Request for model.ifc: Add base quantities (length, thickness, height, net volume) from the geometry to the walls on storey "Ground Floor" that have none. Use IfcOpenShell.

First a look at what the model holds.

```python
import ifcopenshell
import ifcopenshell.util.element
import ifcopenshell.util.unit

model = ifcopenshell.open("model.ifc")
print(model.schema)
for unit_type in ("LENGTHUNIT", "AREAUNIT", "VOLUMEUNIT"):
    print(unit_type, ifcopenshell.util.unit.calculate_unit_scale(model, unit_type))
storey = next(s for s in model.by_type("IfcBuildingStorey") if s.Name == "Ground Floor")
walls = [e for e in ifcopenshell.util.element.get_decomposition(storey) if e.is_a("IfcWall")]
for e in sorted(walls, key=lambda e: e.id()):
    print(e.id(), e.is_a(), e.Name, list(ifcopenshell.util.element.get_psets(e, qtos_only=True)), sep=" | ")
```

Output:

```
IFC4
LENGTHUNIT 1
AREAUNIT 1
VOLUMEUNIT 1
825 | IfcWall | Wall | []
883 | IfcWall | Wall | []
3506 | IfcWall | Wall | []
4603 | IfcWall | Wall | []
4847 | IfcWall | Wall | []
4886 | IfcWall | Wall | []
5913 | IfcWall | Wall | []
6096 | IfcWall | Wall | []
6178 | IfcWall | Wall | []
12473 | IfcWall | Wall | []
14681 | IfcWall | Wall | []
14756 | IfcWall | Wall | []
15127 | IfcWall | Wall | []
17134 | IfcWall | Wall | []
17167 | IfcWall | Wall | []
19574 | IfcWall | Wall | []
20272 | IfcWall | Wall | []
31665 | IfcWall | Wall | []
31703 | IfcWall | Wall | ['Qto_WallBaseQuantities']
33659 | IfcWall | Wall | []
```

```python
import ifcopenshell
import ifcopenshell.api.pset
import ifcopenshell.geom
import ifcopenshell.util.element
import ifcopenshell.util.shape
import ifcopenshell.util.unit

model = ifcopenshell.open("model.ifc")
unit_scale = ifcopenshell.util.unit.calculate_unit_scale(model)
volume_scale = ifcopenshell.util.unit.calculate_unit_scale(model, "VOLUMEUNIT")
settings = ifcopenshell.geom.settings()

storey = next(s for s in model.by_type("IfcBuildingStorey") if s.Name == "Ground Floor")
walls = [e for e in ifcopenshell.util.element.get_decomposition(storey) if e.is_a("IfcWall")]

for e in sorted(walls, key=lambda e: e.id()):
    if ifcopenshell.util.element.get_psets(e, qtos_only=True, should_inherit=False):
        continue
    # Geometry comes back in metres, in the element's own axes.
    shape = ifcopenshell.geom.create_shape(settings, e)
    values = {
        "Length": ifcopenshell.util.shape.get_x(shape.geometry) / unit_scale,
        "Width": ifcopenshell.util.shape.get_y(shape.geometry) / unit_scale,
        "Height": ifcopenshell.util.shape.get_z(shape.geometry) / unit_scale,
        "NetVolume": ifcopenshell.util.shape.get_volume(shape.geometry) / volume_scale,
    }
    qto = ifcopenshell.api.pset.add_qto(model, product=e, name="Qto_WallBaseQuantities")
    ifcopenshell.api.pset.edit_qto(model, qto=qto, properties=values)
    print(e.id(), {k: round(v, 3) for k, v in values.items()})

model.write("model_v2.ifc")
```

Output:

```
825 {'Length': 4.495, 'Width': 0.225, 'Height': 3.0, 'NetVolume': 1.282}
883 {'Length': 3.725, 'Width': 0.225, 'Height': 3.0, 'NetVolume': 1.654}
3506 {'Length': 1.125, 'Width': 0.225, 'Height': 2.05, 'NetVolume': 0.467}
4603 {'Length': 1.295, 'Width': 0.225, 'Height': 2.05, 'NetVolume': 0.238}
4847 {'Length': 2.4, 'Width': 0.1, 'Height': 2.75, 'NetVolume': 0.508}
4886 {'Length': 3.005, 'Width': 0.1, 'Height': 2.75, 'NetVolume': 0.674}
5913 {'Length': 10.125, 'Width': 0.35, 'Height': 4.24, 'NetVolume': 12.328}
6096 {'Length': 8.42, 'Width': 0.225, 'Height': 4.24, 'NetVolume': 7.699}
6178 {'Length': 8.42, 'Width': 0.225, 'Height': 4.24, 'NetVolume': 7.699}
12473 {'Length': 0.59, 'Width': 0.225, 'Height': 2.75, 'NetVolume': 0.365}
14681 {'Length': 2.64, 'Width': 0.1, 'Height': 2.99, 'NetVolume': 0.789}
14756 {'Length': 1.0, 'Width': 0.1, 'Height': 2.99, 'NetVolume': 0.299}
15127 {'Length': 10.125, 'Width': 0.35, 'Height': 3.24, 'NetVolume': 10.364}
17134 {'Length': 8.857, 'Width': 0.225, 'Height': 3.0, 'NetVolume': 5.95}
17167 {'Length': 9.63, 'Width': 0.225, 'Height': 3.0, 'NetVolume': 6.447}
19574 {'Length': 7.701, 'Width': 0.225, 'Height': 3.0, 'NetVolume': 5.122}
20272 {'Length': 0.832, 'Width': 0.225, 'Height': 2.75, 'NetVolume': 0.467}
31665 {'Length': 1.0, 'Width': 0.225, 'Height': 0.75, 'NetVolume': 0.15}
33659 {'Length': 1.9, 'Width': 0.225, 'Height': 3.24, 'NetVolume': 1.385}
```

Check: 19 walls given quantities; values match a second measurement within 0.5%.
